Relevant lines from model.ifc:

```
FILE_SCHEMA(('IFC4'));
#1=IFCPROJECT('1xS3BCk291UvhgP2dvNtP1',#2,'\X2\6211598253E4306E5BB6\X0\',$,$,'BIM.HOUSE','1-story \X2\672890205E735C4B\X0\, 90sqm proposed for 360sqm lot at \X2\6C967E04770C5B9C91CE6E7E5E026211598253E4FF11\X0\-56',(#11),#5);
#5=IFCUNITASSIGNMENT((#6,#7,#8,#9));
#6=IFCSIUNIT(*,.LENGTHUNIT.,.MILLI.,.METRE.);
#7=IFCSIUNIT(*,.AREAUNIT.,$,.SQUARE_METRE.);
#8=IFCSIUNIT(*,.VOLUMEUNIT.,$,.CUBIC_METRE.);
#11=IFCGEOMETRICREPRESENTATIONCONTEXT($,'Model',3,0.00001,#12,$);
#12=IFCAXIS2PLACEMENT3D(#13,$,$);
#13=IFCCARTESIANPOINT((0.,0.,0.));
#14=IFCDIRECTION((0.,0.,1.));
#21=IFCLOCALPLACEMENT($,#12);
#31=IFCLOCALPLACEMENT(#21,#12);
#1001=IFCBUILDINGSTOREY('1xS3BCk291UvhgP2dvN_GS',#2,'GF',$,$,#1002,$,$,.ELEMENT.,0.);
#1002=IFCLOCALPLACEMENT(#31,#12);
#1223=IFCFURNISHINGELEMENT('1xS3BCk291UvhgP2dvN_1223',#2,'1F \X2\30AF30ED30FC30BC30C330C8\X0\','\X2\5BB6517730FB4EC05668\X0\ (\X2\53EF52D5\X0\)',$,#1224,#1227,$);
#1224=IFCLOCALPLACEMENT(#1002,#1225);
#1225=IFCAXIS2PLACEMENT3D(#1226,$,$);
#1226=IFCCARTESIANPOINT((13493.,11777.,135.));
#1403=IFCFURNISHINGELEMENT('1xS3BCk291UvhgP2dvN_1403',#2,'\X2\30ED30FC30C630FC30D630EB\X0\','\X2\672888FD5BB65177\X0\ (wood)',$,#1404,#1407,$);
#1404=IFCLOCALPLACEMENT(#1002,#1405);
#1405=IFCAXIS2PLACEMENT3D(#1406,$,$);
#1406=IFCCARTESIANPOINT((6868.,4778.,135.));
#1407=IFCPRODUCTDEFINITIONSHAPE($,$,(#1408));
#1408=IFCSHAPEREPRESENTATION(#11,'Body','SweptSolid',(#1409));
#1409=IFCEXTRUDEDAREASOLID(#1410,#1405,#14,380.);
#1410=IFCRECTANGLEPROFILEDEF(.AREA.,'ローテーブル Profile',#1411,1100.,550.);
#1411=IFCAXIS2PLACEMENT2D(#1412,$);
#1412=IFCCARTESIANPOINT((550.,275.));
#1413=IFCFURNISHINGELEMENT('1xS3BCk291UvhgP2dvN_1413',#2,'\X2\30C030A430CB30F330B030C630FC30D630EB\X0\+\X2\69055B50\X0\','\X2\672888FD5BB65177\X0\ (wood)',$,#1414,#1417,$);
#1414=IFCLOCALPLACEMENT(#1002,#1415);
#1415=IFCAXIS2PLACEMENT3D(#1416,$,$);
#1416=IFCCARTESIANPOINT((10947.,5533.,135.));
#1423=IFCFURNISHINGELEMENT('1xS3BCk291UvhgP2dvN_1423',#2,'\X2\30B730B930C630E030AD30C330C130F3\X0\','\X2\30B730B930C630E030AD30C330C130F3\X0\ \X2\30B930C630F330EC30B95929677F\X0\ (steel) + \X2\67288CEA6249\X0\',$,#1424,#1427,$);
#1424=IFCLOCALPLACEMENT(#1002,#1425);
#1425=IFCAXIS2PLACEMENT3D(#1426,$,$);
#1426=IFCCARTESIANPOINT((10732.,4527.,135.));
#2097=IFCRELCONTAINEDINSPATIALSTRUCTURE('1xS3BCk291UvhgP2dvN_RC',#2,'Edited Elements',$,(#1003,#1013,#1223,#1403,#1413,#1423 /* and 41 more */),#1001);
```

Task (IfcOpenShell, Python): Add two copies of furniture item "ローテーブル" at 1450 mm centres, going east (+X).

```python
import numpy as np
import ifcopenshell
import ifcopenshell.api.geometry
import ifcopenshell.api.root
import ifcopenshell.util.element
import ifcopenshell.util.placement
import ifcopenshell.util.unit

model = ifcopenshell.open("model.ifc")
unit_scale = ifcopenshell.util.unit.calculate_unit_scale(model)


def reuse_history(source, copy):
    """copy_class also copies each property set's owner history, people and application; keep the originals."""
    for rel in copy.IsDefinedBy:
        if rel.is_a("IfcRelDefinesByProperties") and (history := rel.RelatingPropertyDefinition.OwnerHistory):
            rel.RelatingPropertyDefinition.OwnerHistory = source.OwnerHistory
            ifcopenshell.util.element.remove_deep2(model, history)


source = model.by_id(1403)
base = ifcopenshell.util.placement.get_local_placement(source.ObjectPlacement)
step = np.array([1.0, 0.0, 0.0]) * 1.45 / unit_scale

for i in range(1, 3):
    copy = ifcopenshell.api.root.copy_class(model, product=source)
    copy.Representation = ifcopenshell.util.element.copy_deep(
        model, source.Representation, exclude=["IfcGeometricRepresentationContext", "IfcRepresentationMap"]
    )
    reuse_history(source, copy)
    matrix = base.copy()
    matrix[:3, 3] += i * step
    print("added at", matrix[:3, 3].round(3) + 0.0)
    ifcopenshell.api.geometry.edit_object_placement(model, product=copy, matrix=matrix, is_si=False)

model.write("model-out.ifc")
```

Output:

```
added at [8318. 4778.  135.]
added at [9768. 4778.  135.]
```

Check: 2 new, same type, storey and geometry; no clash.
